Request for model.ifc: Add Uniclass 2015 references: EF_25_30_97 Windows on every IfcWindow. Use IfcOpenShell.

First a look at what the model holds.

```python
import ifcopenshell

model = ifcopenshell.open("model.ifc")
print(model.schema)
print("classifications:", [c.Name for c in model.by_type("IfcClassification")])
for ifc_class in ("IfcDoor", "IfcRoof", "IfcStair", "IfcWall", "IfcWindow"):
    print(ifc_class, len(model.by_type(ifc_class)))
```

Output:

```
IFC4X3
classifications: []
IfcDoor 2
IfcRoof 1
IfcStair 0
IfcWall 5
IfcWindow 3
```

```python
import ifcopenshell
import ifcopenshell.api.classification

model = ifcopenshell.open("model.ifc")

system = ifcopenshell.api.classification.add_classification(model, classification="Uniclass 2015")

codes = {
    "IfcWindow": ("EF_25_30_97", "Windows"),
}
for ifc_class, (code, name) in codes.items():
    products = model.by_type(ifc_class)
    ifcopenshell.api.classification.add_reference(
        model, products=products, classification=system, identification=code, name=name
    )
    print(code, len(products))

model.write("model_rev.ifc")
```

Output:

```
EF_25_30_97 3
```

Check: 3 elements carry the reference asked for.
